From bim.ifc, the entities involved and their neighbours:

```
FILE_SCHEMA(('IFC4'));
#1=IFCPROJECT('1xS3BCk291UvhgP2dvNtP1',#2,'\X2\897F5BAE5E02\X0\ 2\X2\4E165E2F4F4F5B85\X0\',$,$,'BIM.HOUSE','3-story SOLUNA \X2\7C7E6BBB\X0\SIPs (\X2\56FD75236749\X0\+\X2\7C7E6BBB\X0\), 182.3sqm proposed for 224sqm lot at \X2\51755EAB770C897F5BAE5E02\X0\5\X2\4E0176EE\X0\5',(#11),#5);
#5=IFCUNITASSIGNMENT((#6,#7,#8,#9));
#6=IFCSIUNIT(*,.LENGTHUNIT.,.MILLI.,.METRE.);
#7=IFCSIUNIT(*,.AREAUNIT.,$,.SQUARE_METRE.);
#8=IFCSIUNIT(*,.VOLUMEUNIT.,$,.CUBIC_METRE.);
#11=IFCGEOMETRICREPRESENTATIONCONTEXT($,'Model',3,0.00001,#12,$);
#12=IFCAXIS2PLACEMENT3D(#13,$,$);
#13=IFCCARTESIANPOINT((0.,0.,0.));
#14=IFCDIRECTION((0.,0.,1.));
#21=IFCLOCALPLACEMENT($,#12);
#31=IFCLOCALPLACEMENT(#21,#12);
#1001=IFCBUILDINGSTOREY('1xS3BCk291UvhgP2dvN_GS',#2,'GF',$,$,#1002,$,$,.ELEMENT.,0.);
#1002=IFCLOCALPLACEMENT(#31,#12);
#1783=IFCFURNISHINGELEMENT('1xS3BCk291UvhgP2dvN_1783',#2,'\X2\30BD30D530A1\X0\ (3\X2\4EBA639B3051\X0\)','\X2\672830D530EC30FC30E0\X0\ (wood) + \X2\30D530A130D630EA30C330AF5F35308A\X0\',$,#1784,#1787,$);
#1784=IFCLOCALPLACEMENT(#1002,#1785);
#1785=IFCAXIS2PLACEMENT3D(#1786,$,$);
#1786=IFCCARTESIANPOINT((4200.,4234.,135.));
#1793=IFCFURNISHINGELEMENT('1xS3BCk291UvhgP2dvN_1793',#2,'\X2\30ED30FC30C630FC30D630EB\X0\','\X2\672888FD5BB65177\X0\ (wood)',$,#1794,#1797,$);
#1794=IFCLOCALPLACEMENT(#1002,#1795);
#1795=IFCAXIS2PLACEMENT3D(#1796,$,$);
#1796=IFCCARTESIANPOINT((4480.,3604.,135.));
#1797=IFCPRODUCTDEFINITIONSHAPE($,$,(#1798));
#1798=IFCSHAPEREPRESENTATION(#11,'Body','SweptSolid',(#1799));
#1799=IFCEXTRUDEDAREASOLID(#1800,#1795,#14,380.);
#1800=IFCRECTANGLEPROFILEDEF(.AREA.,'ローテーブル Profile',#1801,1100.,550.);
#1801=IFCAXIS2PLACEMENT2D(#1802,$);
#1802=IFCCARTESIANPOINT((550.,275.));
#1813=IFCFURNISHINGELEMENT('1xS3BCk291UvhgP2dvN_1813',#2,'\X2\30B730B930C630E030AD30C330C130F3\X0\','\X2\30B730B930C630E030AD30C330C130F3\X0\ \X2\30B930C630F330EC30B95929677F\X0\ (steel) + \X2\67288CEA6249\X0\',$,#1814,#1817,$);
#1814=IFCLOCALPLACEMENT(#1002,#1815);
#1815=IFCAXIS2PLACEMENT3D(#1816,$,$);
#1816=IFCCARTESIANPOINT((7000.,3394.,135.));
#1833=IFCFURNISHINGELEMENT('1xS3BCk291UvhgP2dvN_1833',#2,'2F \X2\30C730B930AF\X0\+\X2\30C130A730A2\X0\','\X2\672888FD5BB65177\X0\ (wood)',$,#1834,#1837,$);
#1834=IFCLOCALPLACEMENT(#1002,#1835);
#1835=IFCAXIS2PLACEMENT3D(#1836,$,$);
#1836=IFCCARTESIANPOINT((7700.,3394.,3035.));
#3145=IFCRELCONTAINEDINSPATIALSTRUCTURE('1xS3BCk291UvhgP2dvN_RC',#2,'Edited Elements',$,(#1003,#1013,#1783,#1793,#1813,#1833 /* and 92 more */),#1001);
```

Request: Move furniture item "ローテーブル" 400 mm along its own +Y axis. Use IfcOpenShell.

```python
import ifcopenshell
import ifcopenshell.api.geometry
import ifcopenshell.util.placement

model = ifcopenshell.open("bim.ifc")

item = model.by_id(1793)
matrix = ifcopenshell.util.placement.get_local_placement(item.ObjectPlacement)
matrix[:3, 3] += matrix[:3, 1] * 400.0
ifcopenshell.api.geometry.edit_object_placement(model, product=item, matrix=matrix, is_si=False)

print(ifcopenshell.util.placement.get_local_placement(item.ObjectPlacement).round(3) + 0.0)

model.write("bim_rev.ifc")
```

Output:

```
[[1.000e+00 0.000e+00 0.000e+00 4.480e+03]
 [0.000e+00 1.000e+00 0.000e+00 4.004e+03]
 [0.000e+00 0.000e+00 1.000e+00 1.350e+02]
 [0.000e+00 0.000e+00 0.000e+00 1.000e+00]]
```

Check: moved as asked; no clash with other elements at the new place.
